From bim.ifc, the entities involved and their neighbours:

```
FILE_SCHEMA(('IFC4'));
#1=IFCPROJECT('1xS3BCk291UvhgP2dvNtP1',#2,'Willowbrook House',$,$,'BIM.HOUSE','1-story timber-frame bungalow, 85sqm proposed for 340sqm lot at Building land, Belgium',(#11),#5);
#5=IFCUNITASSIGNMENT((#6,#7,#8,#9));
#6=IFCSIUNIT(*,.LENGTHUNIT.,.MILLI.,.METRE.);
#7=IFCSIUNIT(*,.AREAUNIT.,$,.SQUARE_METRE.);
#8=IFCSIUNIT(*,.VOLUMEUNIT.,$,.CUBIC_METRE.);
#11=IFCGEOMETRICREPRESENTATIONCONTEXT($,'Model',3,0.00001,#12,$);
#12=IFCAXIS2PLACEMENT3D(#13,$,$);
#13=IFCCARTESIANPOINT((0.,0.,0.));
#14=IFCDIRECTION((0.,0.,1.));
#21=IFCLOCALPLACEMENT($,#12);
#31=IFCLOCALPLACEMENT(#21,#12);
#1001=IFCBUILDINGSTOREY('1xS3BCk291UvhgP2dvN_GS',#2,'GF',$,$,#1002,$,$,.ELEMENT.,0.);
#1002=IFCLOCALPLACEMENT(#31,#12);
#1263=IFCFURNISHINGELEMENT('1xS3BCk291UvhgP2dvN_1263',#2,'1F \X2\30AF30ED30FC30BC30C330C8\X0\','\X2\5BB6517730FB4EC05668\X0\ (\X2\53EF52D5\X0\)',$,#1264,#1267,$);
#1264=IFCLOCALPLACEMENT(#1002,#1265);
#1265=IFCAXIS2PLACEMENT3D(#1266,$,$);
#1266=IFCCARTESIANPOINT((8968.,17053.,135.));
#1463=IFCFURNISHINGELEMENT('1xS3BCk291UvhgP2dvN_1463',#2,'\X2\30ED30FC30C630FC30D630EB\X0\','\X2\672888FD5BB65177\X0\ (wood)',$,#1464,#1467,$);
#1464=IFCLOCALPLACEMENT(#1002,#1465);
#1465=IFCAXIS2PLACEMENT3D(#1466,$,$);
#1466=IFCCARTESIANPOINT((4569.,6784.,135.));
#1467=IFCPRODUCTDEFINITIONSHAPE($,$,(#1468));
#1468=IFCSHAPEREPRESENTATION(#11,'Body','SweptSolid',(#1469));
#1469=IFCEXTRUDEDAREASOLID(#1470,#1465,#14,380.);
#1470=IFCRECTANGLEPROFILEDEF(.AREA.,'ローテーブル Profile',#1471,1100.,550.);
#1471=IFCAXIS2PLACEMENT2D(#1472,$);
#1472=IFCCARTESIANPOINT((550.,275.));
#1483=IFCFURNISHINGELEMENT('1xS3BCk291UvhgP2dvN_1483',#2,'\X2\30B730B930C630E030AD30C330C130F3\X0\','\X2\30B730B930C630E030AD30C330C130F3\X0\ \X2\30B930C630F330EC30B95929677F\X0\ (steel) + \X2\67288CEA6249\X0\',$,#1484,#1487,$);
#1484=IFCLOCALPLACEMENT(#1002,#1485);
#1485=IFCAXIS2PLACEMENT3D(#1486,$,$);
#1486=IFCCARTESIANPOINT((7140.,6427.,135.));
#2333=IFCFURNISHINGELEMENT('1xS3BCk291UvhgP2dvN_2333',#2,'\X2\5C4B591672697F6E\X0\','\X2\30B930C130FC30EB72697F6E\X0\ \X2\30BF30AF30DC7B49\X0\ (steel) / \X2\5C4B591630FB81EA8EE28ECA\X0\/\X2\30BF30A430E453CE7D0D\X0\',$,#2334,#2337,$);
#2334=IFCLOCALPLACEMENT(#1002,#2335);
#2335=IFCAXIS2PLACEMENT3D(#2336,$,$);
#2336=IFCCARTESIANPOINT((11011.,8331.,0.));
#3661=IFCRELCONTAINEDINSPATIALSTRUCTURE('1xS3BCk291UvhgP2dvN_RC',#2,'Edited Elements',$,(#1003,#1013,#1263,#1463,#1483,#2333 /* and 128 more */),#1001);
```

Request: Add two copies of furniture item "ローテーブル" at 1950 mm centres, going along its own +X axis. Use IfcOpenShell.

```python
import ifcopenshell
import ifcopenshell.api.geometry
import ifcopenshell.api.root
import ifcopenshell.util.element
import ifcopenshell.util.placement
import ifcopenshell.util.unit

model = ifcopenshell.open("bim.ifc")
unit_scale = ifcopenshell.util.unit.calculate_unit_scale(model)


def reuse_history(source, copy):
    """copy_class also copies each property set's owner history, people and application; keep the originals."""
    for rel in copy.IsDefinedBy:
        if rel.is_a("IfcRelDefinesByProperties") and (history := rel.RelatingPropertyDefinition.OwnerHistory):
            rel.RelatingPropertyDefinition.OwnerHistory = source.OwnerHistory
            ifcopenshell.util.element.remove_deep2(model, history)


source = model.by_id(1463)
base = ifcopenshell.util.placement.get_local_placement(source.ObjectPlacement)
step = base[:3, 0] * 1.95 / unit_scale

for i in range(1, 3):
    copy = ifcopenshell.api.root.copy_class(model, product=source)
    copy.Representation = ifcopenshell.util.element.copy_deep(
        model, source.Representation, exclude=["IfcGeometricRepresentationContext", "IfcRepresentationMap"]
    )
    reuse_history(source, copy)
    matrix = base.copy()
    matrix[:3, 3] += i * step
    print("added at", matrix[:3, 3].round(3) + 0.0)
    ifcopenshell.api.geometry.edit_object_placement(model, product=copy, matrix=matrix, is_si=False)

model.write("bim-out.ifc")
```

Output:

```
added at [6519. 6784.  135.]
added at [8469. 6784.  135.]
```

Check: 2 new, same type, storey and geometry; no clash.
